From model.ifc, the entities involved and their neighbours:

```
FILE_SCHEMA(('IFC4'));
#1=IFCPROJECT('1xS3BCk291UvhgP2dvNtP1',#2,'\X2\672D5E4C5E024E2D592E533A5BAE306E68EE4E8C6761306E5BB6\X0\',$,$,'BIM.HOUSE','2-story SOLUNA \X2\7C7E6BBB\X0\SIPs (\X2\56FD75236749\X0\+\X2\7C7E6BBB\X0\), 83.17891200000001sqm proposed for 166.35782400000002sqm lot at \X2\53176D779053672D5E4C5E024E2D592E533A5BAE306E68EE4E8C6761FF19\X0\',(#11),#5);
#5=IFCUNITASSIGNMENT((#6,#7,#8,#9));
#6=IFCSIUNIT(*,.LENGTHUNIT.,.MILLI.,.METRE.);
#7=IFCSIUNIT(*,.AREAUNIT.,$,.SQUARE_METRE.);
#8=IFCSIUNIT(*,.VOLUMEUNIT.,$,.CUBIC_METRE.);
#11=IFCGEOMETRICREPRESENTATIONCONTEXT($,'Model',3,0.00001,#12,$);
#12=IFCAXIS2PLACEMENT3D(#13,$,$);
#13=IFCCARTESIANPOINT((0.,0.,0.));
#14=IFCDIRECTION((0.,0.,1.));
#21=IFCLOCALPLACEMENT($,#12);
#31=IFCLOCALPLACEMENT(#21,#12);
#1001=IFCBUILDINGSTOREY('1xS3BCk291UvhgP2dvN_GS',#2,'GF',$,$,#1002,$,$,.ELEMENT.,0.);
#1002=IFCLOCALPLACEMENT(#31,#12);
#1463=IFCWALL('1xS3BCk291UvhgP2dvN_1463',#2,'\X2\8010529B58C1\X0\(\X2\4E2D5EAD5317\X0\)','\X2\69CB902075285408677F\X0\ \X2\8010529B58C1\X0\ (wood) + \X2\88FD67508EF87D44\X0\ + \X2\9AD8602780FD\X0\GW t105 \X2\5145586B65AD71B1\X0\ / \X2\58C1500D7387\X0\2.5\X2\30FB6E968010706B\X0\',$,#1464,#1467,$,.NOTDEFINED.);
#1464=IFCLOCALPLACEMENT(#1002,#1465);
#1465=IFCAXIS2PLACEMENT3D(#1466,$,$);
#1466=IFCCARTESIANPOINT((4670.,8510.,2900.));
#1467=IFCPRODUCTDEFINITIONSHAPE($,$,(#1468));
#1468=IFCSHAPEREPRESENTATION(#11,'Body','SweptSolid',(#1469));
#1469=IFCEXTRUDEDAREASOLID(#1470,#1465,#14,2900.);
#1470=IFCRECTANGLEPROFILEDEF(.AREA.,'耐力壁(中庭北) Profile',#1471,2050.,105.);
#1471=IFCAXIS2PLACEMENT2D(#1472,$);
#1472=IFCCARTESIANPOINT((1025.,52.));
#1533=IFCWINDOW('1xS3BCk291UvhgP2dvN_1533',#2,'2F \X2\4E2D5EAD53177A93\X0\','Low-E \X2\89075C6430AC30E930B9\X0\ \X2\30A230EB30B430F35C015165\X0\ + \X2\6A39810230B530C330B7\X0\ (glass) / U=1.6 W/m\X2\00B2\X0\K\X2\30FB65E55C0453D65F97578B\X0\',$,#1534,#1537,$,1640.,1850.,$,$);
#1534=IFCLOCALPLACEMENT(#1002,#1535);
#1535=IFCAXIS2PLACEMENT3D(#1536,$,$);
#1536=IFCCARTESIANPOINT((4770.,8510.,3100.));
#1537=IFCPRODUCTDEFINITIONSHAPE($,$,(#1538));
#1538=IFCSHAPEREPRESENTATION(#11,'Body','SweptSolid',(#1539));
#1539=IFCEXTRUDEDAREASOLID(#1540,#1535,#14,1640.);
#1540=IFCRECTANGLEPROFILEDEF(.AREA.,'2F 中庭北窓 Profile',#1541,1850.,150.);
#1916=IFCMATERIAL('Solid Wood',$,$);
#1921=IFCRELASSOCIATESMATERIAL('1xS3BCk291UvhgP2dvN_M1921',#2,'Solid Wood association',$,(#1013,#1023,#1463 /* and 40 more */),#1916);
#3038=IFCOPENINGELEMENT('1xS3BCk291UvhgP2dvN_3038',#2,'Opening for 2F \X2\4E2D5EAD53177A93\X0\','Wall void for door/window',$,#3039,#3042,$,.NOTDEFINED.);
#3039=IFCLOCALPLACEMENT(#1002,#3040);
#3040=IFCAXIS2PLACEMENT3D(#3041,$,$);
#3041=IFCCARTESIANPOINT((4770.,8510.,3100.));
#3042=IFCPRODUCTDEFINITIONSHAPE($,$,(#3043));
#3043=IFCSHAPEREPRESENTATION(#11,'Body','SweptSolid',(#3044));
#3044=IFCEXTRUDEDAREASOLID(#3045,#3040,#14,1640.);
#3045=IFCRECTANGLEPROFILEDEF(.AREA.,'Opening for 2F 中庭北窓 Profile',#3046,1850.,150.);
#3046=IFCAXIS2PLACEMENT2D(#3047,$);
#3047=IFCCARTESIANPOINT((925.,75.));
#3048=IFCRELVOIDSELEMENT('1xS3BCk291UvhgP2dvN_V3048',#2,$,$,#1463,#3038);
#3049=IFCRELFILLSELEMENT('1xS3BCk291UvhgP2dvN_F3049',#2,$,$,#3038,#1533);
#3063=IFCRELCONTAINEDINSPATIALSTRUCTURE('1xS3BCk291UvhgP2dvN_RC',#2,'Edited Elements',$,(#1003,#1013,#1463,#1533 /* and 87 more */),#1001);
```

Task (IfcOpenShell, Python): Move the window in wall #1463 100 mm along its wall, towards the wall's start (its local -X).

```python
import ifcopenshell
import ifcopenshell.api.geometry
import ifcopenshell.util.placement
import ifcopenshell.util.unit

model = ifcopenshell.open("model.ifc")
unit_scale = ifcopenshell.util.unit.calculate_unit_scale(model)

window = model.by_id(1533)
opening = window.FillsVoids[0].RelatingOpeningElement
wall = opening.VoidsElements[0].RelatingBuildingElement

wall_matrix = ifcopenshell.util.placement.get_local_placement(wall.ObjectPlacement)
shift = wall_matrix[:3, 0] * -0.1 / unit_scale
before = ifcopenshell.util.placement.get_local_placement(window.ObjectPlacement)[:3, 3].copy()

# The window is not placed relative to its opening, so move both.
for product in (opening, window):
    matrix = ifcopenshell.util.placement.get_local_placement(product.ObjectPlacement)
    matrix[:3, 3] += shift
    ifcopenshell.api.geometry.edit_object_placement(model, product=product, matrix=matrix, is_si=False)

after = ifcopenshell.util.placement.get_local_placement(window.ObjectPlacement)[:3, 3]
print("window moved by", (after - before).round(3) + 0.0)

model.write("model_updated.ifc")
```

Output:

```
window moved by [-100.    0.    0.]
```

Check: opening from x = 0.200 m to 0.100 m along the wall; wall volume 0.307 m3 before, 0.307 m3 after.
